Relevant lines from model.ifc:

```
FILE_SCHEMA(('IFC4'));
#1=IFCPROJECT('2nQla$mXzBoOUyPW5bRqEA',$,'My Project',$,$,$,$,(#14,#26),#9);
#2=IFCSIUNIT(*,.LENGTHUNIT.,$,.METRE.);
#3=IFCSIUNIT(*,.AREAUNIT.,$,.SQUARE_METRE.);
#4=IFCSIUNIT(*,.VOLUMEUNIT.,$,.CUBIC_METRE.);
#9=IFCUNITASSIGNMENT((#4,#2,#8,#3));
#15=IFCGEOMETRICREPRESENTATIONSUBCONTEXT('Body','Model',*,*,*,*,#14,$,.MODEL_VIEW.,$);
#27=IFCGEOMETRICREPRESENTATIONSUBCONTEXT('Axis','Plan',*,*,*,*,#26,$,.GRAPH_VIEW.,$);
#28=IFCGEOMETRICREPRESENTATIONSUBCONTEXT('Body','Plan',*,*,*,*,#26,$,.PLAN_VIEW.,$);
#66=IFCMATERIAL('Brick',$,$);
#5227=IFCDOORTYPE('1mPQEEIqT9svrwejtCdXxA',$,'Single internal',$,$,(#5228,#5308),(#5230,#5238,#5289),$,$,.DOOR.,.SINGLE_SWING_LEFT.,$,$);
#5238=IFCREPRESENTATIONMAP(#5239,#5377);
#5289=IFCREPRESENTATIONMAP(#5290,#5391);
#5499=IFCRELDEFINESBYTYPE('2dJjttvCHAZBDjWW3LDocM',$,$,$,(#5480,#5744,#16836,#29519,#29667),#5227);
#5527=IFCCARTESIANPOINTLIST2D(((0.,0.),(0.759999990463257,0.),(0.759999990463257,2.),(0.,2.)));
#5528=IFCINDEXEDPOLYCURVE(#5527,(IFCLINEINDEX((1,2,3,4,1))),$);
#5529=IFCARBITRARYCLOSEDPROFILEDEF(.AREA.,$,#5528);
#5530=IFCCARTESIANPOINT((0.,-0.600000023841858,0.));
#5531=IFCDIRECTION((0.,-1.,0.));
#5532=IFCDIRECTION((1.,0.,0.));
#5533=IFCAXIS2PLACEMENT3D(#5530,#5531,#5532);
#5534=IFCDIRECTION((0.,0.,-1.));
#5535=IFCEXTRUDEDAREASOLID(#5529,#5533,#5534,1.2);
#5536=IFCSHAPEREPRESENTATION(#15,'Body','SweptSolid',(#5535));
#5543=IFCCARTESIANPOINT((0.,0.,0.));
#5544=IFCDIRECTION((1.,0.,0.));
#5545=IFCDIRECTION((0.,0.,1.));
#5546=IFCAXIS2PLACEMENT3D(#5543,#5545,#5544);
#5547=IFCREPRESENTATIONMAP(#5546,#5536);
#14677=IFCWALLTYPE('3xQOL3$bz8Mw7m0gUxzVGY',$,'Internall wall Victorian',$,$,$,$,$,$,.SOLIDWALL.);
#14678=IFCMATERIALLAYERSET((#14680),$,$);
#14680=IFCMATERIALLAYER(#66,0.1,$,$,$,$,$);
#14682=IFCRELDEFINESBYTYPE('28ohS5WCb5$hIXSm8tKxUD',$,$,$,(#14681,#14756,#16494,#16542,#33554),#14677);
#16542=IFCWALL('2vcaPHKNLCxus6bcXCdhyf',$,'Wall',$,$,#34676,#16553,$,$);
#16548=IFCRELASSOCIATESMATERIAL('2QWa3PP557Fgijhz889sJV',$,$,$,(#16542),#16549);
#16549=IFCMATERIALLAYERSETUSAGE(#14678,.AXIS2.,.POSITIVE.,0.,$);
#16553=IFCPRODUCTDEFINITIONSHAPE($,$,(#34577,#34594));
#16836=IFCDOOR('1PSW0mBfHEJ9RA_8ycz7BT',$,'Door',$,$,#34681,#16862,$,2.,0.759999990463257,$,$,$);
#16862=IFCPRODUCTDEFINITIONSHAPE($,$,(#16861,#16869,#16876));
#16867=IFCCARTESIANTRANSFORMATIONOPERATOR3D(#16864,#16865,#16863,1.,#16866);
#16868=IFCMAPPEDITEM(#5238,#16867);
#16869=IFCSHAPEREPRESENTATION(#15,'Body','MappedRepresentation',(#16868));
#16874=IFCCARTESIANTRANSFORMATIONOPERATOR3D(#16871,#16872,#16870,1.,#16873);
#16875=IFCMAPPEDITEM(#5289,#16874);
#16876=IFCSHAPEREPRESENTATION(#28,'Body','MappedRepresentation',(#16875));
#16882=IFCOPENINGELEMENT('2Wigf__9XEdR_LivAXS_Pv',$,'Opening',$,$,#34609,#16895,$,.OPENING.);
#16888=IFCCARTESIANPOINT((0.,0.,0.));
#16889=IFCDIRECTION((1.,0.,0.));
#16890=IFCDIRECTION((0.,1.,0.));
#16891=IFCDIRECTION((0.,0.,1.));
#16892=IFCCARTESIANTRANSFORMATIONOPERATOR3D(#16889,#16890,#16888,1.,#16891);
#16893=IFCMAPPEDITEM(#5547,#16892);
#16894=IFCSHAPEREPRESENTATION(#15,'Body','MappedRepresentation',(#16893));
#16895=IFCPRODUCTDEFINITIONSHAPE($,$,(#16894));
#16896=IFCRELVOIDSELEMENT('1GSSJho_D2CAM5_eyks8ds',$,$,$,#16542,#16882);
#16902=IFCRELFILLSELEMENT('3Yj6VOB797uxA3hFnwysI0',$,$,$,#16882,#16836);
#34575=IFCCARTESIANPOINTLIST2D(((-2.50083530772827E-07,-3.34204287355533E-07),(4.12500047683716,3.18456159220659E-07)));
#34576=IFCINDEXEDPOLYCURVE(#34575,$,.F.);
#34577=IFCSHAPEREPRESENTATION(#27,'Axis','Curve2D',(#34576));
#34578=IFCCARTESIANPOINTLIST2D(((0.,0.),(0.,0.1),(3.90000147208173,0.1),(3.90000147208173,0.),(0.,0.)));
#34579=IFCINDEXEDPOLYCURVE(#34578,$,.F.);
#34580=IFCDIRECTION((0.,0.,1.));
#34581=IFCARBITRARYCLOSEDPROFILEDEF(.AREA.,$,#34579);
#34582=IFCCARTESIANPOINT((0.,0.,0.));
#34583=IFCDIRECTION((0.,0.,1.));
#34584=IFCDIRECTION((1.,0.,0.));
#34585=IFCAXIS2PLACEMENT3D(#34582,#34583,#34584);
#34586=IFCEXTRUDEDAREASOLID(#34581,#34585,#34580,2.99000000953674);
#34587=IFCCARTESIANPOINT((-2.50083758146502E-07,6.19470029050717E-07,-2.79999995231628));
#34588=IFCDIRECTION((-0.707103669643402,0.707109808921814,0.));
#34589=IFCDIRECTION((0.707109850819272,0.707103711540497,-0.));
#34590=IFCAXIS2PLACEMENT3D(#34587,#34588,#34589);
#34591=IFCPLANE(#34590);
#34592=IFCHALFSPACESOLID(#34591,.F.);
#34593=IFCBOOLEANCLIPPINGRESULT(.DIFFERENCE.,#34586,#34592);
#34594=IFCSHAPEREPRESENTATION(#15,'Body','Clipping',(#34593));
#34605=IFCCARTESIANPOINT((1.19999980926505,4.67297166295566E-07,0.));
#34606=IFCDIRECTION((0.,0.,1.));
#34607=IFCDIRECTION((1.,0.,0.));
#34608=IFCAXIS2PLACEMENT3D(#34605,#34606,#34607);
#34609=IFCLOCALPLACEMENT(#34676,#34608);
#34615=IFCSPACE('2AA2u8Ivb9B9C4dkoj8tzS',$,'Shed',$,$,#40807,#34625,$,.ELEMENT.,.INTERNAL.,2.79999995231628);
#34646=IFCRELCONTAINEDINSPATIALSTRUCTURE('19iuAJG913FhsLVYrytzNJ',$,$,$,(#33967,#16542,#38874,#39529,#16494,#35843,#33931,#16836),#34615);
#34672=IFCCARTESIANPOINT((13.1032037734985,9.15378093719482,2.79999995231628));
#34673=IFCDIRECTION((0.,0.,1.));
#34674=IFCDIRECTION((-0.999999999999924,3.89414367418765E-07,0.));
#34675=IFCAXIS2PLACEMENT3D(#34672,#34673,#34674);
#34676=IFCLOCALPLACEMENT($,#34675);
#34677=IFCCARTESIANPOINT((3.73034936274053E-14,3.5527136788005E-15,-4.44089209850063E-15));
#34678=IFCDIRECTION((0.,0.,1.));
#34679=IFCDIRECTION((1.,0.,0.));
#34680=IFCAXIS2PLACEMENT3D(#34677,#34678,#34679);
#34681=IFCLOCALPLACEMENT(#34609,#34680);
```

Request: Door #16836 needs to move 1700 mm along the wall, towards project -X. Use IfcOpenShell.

```python
import ifcopenshell
import ifcopenshell.api.geometry
import ifcopenshell.util.placement
import ifcopenshell.util.unit

model = ifcopenshell.open("model.ifc")
unit_scale = ifcopenshell.util.unit.calculate_unit_scale(model)

door = model.by_guid("1PSW0mBfHEJ9RA_8ycz7BT")
opening = door.FillsVoids[0].RelatingOpeningElement
wall = opening.VoidsElements[0].RelatingBuildingElement

wall_matrix = ifcopenshell.util.placement.get_local_placement(wall.ObjectPlacement)
shift = wall_matrix[:3, 0] * 1.7 / unit_scale
before = ifcopenshell.util.placement.get_local_placement(door.ObjectPlacement)[:3, 3].copy()

# The door is placed relative to its opening, so it follows when the opening moves.
matrix = ifcopenshell.util.placement.get_local_placement(opening.ObjectPlacement)
matrix[:3, 3] += shift
ifcopenshell.api.geometry.edit_object_placement(
    model, product=opening, matrix=matrix, is_si=False, should_transform_children=True
)

after = ifcopenshell.util.placement.get_local_placement(door.ObjectPlacement)[:3, 3]
print("door moved by", (after - before).round(3) + 0.0)

model.write("model-out.ifc")
```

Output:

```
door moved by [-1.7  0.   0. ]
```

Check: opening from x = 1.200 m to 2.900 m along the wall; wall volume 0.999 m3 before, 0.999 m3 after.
